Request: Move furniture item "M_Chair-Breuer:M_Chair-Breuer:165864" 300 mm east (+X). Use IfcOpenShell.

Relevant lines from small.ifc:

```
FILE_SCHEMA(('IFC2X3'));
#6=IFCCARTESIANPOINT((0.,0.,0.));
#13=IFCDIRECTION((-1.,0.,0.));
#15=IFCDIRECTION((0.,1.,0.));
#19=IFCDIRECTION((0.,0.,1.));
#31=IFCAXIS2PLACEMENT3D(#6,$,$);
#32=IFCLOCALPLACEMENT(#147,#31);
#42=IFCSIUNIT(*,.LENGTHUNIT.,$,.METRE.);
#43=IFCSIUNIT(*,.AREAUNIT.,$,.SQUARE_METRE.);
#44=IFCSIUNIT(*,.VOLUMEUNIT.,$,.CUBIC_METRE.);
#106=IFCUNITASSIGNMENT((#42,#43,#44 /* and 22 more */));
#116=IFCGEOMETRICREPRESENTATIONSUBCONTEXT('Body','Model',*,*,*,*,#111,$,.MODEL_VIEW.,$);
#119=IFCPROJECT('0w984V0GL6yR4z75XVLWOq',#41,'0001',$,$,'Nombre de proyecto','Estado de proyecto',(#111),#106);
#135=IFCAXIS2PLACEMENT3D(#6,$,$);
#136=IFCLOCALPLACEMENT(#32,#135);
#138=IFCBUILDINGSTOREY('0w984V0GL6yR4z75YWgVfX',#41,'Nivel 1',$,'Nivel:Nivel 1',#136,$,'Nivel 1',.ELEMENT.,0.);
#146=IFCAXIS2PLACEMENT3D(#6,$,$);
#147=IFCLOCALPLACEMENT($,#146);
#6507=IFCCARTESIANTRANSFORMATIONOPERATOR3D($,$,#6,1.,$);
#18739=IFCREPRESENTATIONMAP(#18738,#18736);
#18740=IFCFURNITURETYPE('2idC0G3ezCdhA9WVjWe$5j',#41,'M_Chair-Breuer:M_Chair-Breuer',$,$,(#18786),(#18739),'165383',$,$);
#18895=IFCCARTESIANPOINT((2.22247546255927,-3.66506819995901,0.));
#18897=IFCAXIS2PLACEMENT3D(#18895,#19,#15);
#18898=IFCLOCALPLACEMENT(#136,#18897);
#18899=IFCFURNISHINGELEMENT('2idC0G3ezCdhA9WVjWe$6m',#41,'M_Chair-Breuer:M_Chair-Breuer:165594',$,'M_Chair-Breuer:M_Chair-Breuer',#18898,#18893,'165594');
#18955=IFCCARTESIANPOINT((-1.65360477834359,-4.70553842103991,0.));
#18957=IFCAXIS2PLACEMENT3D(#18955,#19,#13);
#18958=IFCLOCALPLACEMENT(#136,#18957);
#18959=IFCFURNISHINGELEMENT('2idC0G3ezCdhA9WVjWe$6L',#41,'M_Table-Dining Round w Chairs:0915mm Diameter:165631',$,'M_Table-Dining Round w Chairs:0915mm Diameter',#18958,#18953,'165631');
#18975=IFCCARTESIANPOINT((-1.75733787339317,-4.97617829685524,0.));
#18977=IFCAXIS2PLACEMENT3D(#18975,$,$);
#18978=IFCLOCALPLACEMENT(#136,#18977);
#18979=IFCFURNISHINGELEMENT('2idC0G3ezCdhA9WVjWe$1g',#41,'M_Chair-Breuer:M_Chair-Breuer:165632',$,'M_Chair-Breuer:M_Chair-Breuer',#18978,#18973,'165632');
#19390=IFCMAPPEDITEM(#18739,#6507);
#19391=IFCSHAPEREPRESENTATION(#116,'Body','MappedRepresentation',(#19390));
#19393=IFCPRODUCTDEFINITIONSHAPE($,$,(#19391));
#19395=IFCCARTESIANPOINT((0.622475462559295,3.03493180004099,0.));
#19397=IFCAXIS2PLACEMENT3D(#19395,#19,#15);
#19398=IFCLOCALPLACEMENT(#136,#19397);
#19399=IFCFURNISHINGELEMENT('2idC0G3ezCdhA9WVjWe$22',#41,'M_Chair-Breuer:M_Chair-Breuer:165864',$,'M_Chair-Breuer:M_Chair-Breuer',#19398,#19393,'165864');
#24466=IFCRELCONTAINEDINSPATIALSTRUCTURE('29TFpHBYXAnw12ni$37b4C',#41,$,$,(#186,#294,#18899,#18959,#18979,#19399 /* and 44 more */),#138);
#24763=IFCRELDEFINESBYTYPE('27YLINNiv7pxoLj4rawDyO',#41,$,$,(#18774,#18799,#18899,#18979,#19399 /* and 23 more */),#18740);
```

```python
import ifcopenshell
import ifcopenshell.api.geometry
import ifcopenshell.util.placement
import ifcopenshell.util.unit

model = ifcopenshell.open("small.ifc")
unit_scale = ifcopenshell.util.unit.calculate_unit_scale(model)

item = model.by_guid("2idC0G3ezCdhA9WVjWe$22")
matrix = ifcopenshell.util.placement.get_local_placement(item.ObjectPlacement)
matrix[0, 3] += 0.3 / unit_scale
ifcopenshell.api.geometry.edit_object_placement(model, product=item, matrix=matrix, is_si=False)

print(ifcopenshell.util.placement.get_local_placement(item.ObjectPlacement).round(3) + 0.0)

model.write("small-out.ifc")
```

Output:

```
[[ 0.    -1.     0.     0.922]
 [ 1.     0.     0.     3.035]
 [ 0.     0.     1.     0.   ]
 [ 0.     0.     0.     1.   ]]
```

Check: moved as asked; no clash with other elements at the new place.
